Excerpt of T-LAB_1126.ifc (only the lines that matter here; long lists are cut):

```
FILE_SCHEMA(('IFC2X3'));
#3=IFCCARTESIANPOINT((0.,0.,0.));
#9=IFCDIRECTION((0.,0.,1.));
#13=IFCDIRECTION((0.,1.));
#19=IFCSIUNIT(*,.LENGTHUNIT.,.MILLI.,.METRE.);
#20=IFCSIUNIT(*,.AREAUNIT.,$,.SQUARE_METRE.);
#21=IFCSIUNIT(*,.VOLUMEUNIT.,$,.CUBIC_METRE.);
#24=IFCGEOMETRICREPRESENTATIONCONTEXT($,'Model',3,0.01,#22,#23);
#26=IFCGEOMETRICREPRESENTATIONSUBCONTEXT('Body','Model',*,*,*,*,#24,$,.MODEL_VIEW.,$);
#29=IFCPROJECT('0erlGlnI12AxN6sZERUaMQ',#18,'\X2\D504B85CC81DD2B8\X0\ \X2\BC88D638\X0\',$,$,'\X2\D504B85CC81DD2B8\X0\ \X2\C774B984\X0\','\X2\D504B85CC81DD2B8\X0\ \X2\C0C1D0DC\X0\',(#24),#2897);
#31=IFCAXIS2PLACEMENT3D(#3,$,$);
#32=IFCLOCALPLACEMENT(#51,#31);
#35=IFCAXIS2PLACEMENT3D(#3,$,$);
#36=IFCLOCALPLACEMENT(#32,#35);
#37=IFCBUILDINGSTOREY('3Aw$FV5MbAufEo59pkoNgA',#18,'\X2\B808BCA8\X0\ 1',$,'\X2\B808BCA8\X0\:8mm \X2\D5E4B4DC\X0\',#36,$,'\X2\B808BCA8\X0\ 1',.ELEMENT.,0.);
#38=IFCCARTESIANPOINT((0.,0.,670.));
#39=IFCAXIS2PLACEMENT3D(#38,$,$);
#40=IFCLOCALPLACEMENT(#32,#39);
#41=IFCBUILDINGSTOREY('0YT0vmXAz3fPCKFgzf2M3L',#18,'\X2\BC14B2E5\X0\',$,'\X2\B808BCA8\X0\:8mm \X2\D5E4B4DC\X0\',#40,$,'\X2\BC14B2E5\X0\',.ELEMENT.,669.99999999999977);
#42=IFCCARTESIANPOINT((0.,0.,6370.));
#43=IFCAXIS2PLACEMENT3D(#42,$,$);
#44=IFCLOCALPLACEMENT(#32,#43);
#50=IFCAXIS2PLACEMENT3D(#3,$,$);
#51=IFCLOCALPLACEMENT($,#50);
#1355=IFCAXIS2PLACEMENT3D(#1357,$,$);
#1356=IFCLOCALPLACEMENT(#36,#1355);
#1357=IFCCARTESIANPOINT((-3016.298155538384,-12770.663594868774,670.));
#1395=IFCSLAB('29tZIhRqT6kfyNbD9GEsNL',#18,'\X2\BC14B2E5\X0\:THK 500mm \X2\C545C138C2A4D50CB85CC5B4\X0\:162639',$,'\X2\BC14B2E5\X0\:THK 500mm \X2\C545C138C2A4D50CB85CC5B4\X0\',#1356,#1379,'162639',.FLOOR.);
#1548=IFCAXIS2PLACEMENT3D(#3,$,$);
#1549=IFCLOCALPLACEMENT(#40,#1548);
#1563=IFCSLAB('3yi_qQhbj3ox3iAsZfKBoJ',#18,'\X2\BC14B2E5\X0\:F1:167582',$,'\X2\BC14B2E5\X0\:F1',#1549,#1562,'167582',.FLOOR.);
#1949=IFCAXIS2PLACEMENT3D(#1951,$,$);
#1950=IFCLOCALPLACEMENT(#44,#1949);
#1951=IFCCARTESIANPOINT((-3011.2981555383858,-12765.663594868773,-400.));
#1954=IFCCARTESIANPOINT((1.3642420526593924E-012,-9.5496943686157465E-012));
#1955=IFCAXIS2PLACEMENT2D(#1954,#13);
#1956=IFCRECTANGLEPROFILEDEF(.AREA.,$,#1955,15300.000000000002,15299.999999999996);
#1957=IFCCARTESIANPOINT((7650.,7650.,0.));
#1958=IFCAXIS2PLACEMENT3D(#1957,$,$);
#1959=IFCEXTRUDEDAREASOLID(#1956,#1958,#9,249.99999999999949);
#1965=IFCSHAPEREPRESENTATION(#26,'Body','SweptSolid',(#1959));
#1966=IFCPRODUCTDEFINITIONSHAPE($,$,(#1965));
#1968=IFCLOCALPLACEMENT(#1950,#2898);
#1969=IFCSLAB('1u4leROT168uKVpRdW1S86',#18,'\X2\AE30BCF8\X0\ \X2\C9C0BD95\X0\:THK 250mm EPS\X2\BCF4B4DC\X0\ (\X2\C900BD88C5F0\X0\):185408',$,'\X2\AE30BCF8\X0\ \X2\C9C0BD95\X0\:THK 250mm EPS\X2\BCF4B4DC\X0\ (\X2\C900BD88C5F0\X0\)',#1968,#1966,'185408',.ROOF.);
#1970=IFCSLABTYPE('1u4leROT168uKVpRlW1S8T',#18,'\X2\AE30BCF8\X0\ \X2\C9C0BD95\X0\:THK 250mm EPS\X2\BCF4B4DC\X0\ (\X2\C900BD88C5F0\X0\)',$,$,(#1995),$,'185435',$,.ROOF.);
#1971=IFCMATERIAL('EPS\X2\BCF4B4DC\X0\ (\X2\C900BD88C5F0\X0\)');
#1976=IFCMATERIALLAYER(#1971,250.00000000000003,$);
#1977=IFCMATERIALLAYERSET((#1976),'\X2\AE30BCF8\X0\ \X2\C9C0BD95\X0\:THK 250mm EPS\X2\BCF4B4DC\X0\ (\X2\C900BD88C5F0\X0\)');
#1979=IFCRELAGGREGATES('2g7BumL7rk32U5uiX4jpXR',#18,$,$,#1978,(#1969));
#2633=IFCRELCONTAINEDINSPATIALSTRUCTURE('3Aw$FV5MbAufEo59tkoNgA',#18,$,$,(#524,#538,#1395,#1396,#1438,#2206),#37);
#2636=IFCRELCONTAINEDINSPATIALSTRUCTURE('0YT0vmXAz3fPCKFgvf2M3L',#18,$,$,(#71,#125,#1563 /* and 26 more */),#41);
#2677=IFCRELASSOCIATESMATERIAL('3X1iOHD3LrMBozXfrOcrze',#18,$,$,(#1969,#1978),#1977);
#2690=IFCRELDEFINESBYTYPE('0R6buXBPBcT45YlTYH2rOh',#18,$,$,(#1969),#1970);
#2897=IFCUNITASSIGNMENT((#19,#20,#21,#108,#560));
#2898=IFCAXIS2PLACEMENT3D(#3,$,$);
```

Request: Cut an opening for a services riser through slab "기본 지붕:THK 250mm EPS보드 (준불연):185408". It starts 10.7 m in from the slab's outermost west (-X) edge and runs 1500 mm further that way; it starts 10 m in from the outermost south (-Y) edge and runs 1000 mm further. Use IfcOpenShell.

```python
import numpy as np
import ifcopenshell
import ifcopenshell.api.feature
import ifcopenshell.api.geometry
import ifcopenshell.api.root
import ifcopenshell.geom
import ifcopenshell.util.placement
import ifcopenshell.util.representation
import ifcopenshell.util.shape
import ifcopenshell.util.unit

model = ifcopenshell.open("T-LAB_1126.ifc")
unit_scale = ifcopenshell.util.unit.calculate_unit_scale(model)
settings = ifcopenshell.geom.settings()


def volume(element):
    """Net volume in cubic metres, openings subtracted."""
    shape = ifcopenshell.geom.create_shape(settings, element)
    return ifcopenshell.util.shape.get_volume(shape.geometry)


slab = model.by_guid("1u4leROT168uKVpRdW1S86")
before = volume(slab)

# Extent in the slab's own axes, in metres. The edges named are its -X and -Y sides.
slab_shape = ifcopenshell.geom.create_shape(settings, slab)
vertices = ifcopenshell.util.shape.get_vertices(slab_shape.geometry)
x_min, y_min, bottom = vertices.min(axis=0)
top = vertices[:, 2].max()

opening = ifcopenshell.api.root.create_entity(model, ifc_class="IfcOpeningElement", name="Services riser opening")
context = ifcopenshell.util.representation.get_context(model, "Model", "Body", "MODEL_VIEW")
width, depth = 1.5, 1
outline = [(0.0, 0.0), (width, 0.0), (width, depth), (0.0, depth), (0.0, 0.0)]
# Overshoot both faces by 50 mm so the cut is clean.
shape = ifcopenshell.api.geometry.add_slab_representation(
    model, context=context, depth=top - bottom + 0.1, polyline=outline
)
ifcopenshell.api.geometry.assign_representation(model, product=opening, representation=shape)

matrix = ifcopenshell.util.placement.get_local_placement(slab.ObjectPlacement)
matrix[:, 3] = matrix @ np.append(np.array([x_min + 10.7, y_min + 10, bottom - 0.05]) / unit_scale, 1.0)
ifcopenshell.api.geometry.edit_object_placement(model, product=opening, matrix=matrix, is_si=False)
ifcopenshell.api.feature.add_feature(model, feature=opening, element=slab)

after = volume(slab)

print(f"slab volume {before:.3f} -> {after:.3f} m3")

model.write("T-LAB_1126-out.ifc")
```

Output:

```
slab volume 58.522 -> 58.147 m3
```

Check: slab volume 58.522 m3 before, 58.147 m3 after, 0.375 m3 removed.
